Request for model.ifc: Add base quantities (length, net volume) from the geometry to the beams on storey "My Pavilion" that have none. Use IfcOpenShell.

First a look at what the model holds.

```python
import ifcopenshell
import ifcopenshell.util.element
import ifcopenshell.util.unit

model = ifcopenshell.open("model.ifc")
print(model.schema)
for unit_type in ("LENGTHUNIT", "AREAUNIT", "VOLUMEUNIT"):
    print(unit_type, ifcopenshell.util.unit.calculate_unit_scale(model, unit_type))
storey = next(s for s in model.by_type("IfcBuildingStorey") if s.Name == "My Pavilion")
beams = [e for e in ifcopenshell.util.element.get_decomposition(storey) if e.is_a("IfcBeam")]
for e in sorted(beams, key=lambda e: e.id()):
    print(e.id(), e.is_a(), e.Name, list(ifcopenshell.util.element.get_psets(e, qtos_only=True)), sep=" | ")
```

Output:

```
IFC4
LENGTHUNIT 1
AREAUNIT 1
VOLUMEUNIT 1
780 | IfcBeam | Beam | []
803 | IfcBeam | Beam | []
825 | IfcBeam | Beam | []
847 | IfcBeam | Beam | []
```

```python
import ifcopenshell
import ifcopenshell.api.pset
import ifcopenshell.geom
import ifcopenshell.util.element
import ifcopenshell.util.shape
import ifcopenshell.util.unit

model = ifcopenshell.open("model.ifc")
unit_scale = ifcopenshell.util.unit.calculate_unit_scale(model)
volume_scale = ifcopenshell.util.unit.calculate_unit_scale(model, "VOLUMEUNIT")
settings = ifcopenshell.geom.settings()

storey = next(s for s in model.by_type("IfcBuildingStorey") if s.Name == "My Pavilion")
beams = [e for e in ifcopenshell.util.element.get_decomposition(storey) if e.is_a("IfcBeam")]

for e in sorted(beams, key=lambda e: e.id()):
    if ifcopenshell.util.element.get_psets(e, qtos_only=True, should_inherit=False):
        continue
    # Geometry comes back in metres, in the element's own axes.
    shape = ifcopenshell.geom.create_shape(settings, e)
    values = {
        "Length": ifcopenshell.util.shape.get_max_xyz(shape.geometry) / unit_scale,
        "NetVolume": ifcopenshell.util.shape.get_volume(shape.geometry) / volume_scale,
    }
    qto = ifcopenshell.api.pset.add_qto(model, product=e, name="Qto_BeamBaseQuantities")
    ifcopenshell.api.pset.edit_qto(model, qto=qto, properties=values)
    print(e.id(), {k: round(v, 3) for k, v in values.items()})

model.write("model_v2.ifc")
```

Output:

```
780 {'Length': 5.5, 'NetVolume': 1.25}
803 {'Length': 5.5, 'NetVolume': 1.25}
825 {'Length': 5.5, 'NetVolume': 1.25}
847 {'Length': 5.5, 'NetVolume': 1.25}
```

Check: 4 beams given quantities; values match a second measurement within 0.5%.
